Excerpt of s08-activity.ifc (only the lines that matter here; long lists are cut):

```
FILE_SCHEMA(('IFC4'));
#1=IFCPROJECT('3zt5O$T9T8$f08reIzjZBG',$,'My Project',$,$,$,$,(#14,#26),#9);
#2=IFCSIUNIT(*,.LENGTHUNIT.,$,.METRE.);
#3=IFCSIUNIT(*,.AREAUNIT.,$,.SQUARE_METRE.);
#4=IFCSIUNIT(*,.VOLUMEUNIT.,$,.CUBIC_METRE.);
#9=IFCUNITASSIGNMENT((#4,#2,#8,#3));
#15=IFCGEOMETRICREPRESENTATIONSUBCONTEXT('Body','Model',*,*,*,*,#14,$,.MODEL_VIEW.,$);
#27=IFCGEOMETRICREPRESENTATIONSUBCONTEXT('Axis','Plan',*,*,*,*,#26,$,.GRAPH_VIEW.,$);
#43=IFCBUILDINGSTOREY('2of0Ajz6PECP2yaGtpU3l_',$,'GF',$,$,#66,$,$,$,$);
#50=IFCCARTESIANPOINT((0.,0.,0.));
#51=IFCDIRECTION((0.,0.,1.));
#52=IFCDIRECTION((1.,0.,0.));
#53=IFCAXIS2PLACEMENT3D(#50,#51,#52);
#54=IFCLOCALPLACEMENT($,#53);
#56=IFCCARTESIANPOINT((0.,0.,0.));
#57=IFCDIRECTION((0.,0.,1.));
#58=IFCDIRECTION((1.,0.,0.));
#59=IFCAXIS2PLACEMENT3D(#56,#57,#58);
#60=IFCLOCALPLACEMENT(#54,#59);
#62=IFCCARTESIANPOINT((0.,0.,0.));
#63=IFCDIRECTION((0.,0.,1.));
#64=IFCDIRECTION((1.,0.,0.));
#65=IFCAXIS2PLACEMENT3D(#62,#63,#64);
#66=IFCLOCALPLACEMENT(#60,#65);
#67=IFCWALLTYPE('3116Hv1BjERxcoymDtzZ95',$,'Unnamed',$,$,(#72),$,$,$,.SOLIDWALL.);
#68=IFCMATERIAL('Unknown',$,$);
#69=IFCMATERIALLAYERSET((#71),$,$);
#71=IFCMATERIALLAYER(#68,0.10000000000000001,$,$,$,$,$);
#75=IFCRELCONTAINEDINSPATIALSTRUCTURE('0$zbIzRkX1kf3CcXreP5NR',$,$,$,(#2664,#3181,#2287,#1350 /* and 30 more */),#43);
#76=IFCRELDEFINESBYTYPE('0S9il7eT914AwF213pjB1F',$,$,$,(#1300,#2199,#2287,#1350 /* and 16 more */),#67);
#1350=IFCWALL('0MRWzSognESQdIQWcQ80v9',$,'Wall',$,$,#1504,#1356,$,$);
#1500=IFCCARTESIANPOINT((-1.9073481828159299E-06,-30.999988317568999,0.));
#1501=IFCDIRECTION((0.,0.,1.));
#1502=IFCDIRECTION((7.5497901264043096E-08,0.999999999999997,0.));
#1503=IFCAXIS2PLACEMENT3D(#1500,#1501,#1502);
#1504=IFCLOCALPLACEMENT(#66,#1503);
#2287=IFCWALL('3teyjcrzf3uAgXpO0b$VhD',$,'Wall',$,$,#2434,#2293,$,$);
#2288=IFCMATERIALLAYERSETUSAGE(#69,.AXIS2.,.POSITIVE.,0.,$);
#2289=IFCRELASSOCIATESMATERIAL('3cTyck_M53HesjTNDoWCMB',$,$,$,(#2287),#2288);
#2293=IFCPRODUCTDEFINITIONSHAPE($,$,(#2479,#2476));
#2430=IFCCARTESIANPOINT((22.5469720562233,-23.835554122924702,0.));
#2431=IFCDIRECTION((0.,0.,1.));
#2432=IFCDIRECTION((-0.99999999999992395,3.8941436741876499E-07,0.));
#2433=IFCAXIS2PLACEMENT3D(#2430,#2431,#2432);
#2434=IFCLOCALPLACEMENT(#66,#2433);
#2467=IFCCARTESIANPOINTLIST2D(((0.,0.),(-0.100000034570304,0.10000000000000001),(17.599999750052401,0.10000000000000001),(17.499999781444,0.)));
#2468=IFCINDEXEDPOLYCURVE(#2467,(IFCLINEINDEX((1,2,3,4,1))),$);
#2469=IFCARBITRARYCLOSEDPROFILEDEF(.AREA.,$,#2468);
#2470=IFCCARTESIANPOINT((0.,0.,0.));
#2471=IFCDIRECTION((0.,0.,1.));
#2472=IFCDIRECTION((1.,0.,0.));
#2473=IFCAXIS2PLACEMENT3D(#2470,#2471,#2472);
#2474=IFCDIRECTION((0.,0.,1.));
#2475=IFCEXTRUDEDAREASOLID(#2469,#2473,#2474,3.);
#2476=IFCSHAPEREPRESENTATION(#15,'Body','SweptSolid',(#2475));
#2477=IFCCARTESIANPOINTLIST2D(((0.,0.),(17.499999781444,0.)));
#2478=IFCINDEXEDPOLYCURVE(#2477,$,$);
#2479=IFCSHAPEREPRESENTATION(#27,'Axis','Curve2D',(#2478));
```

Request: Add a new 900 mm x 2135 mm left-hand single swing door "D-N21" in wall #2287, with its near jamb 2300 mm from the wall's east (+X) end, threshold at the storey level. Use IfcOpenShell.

```python
import numpy as np
import ifcopenshell
import ifcopenshell.api.feature
import ifcopenshell.api.geometry
import ifcopenshell.api.root
import ifcopenshell.api.spatial
import ifcopenshell.geom
import ifcopenshell.util.element
import ifcopenshell.util.placement
import ifcopenshell.util.representation
import ifcopenshell.util.shape
import ifcopenshell.util.unit

model = ifcopenshell.open("s08-activity.ifc")
unit_scale = ifcopenshell.util.unit.calculate_unit_scale(model)
settings = ifcopenshell.geom.settings()


def volume(element):
    """Net volume in cubic metres, openings subtracted."""
    shape = ifcopenshell.geom.create_shape(settings, element)
    return ifcopenshell.util.shape.get_volume(shape.geometry)


wall = model.by_id(2287)
storey = ifcopenshell.util.element.get_container(wall, ifc_class="IfcBuildingStorey")
context = ifcopenshell.util.representation.get_context(model, "Model", "Body", "MODEL_VIEW")
before = volume(wall)

width, height, from_end, sill = 0.9, 2.135, 2.3, 0.0  # metres

# The wall runs along its own X axis, and the end named is its -X end.
wall_shape = ifcopenshell.geom.create_shape(settings, wall)
x, y, z = ifcopenshell.util.shape.get_vertices(wall_shape.geometry).T
start = x.min() + from_end
face, thickness = float(y.min()), float(y.max() - y.min())
wall_matrix = ifcopenshell.util.placement.get_local_placement(wall.ObjectPlacement)
level = ifcopenshell.util.placement.get_local_placement(storey.ObjectPlacement)[2, 3]


def in_wall(x, y):
    """Placement at x, y metres in the wall's axes, at sill height."""
    matrix = wall_matrix.copy()
    matrix[:, 3] = wall_matrix @ np.array([x / unit_scale, y / unit_scale, 0.0, 1.0])
    matrix[2, 3] = level + sill / unit_scale
    return matrix


# Opening: a box that overshoots both wall faces by 50 mm.
opening = ifcopenshell.api.root.create_entity(model, ifc_class="IfcOpeningElement", predefined_type="OPENING")
box = ifcopenshell.api.geometry.add_wall_representation(
    model, context=context, length=width, height=height, thickness=thickness + 0.1
)
ifcopenshell.api.geometry.assign_representation(model, product=opening, representation=box)
ifcopenshell.api.geometry.edit_object_placement(model, product=opening, matrix=in_wall(start, face - 0.05), is_si=False)
ifcopenshell.api.feature.add_feature(model, feature=opening, element=wall)

door = ifcopenshell.api.root.create_entity(model, ifc_class="IfcDoor", name="D-N21", predefined_type="DOOR")
door.OverallWidth, door.OverallHeight = width / unit_scale, height / unit_scale
door.OperationType = "SINGLE_SWING_LEFT"
body = ifcopenshell.api.geometry.add_door_representation(
    model,
    context=context,
    overall_width=door.OverallWidth,
    overall_height=door.OverallHeight,
    operation_type="SINGLE_SWING_LEFT",
    lining_properties={"LiningDepth": thickness / unit_scale, "ThresholdDepth": thickness / unit_scale},
)
ifcopenshell.api.geometry.assign_representation(model, product=door, representation=body)
ifcopenshell.api.spatial.assign_container(model, products=[door], relating_structure=storey)
ifcopenshell.api.feature.add_filling(model, opening=opening, element=door)

# The lining spans the wall, so the door starts at the wall face.
ifcopenshell.api.geometry.edit_object_placement(model, product=door, matrix=in_wall(start, face), is_si=False)

after = volume(wall)

print(f"wall volume {before:.3f} -> {after:.3f} m3")

model.write("s08-activity_v2.ifc")
```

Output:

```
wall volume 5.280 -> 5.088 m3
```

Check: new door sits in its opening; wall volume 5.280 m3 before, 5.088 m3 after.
